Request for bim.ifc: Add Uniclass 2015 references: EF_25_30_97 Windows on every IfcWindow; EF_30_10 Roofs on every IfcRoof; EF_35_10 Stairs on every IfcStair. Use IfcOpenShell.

First a look at what the model holds.

```python
import ifcopenshell

model = ifcopenshell.open("bim.ifc")
print(model.schema)
print("classifications:", [c.Name for c in model.by_type("IfcClassification")])
for ifc_class in ("IfcDoor", "IfcRoof", "IfcStair", "IfcWall", "IfcWindow"):
    print(ifc_class, len(model.by_type(ifc_class)))
```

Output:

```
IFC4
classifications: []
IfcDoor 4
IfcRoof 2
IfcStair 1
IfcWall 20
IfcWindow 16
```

```python
import ifcopenshell
import ifcopenshell.api.classification

model = ifcopenshell.open("bim.ifc")

system = ifcopenshell.api.classification.add_classification(model, classification="Uniclass 2015")

codes = {
    "IfcWindow": ("EF_25_30_97", "Windows"),
    "IfcRoof": ("EF_30_10", "Roofs"),
    "IfcStair": ("EF_35_10", "Stairs"),
}
for ifc_class, (code, name) in codes.items():
    products = model.by_type(ifc_class)
    ifcopenshell.api.classification.add_reference(
        model, products=products, classification=system, identification=code, name=name
    )
    print(code, len(products))

model.write("bim_v2.ifc")
```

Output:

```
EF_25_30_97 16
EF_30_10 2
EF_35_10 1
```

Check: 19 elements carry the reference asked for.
